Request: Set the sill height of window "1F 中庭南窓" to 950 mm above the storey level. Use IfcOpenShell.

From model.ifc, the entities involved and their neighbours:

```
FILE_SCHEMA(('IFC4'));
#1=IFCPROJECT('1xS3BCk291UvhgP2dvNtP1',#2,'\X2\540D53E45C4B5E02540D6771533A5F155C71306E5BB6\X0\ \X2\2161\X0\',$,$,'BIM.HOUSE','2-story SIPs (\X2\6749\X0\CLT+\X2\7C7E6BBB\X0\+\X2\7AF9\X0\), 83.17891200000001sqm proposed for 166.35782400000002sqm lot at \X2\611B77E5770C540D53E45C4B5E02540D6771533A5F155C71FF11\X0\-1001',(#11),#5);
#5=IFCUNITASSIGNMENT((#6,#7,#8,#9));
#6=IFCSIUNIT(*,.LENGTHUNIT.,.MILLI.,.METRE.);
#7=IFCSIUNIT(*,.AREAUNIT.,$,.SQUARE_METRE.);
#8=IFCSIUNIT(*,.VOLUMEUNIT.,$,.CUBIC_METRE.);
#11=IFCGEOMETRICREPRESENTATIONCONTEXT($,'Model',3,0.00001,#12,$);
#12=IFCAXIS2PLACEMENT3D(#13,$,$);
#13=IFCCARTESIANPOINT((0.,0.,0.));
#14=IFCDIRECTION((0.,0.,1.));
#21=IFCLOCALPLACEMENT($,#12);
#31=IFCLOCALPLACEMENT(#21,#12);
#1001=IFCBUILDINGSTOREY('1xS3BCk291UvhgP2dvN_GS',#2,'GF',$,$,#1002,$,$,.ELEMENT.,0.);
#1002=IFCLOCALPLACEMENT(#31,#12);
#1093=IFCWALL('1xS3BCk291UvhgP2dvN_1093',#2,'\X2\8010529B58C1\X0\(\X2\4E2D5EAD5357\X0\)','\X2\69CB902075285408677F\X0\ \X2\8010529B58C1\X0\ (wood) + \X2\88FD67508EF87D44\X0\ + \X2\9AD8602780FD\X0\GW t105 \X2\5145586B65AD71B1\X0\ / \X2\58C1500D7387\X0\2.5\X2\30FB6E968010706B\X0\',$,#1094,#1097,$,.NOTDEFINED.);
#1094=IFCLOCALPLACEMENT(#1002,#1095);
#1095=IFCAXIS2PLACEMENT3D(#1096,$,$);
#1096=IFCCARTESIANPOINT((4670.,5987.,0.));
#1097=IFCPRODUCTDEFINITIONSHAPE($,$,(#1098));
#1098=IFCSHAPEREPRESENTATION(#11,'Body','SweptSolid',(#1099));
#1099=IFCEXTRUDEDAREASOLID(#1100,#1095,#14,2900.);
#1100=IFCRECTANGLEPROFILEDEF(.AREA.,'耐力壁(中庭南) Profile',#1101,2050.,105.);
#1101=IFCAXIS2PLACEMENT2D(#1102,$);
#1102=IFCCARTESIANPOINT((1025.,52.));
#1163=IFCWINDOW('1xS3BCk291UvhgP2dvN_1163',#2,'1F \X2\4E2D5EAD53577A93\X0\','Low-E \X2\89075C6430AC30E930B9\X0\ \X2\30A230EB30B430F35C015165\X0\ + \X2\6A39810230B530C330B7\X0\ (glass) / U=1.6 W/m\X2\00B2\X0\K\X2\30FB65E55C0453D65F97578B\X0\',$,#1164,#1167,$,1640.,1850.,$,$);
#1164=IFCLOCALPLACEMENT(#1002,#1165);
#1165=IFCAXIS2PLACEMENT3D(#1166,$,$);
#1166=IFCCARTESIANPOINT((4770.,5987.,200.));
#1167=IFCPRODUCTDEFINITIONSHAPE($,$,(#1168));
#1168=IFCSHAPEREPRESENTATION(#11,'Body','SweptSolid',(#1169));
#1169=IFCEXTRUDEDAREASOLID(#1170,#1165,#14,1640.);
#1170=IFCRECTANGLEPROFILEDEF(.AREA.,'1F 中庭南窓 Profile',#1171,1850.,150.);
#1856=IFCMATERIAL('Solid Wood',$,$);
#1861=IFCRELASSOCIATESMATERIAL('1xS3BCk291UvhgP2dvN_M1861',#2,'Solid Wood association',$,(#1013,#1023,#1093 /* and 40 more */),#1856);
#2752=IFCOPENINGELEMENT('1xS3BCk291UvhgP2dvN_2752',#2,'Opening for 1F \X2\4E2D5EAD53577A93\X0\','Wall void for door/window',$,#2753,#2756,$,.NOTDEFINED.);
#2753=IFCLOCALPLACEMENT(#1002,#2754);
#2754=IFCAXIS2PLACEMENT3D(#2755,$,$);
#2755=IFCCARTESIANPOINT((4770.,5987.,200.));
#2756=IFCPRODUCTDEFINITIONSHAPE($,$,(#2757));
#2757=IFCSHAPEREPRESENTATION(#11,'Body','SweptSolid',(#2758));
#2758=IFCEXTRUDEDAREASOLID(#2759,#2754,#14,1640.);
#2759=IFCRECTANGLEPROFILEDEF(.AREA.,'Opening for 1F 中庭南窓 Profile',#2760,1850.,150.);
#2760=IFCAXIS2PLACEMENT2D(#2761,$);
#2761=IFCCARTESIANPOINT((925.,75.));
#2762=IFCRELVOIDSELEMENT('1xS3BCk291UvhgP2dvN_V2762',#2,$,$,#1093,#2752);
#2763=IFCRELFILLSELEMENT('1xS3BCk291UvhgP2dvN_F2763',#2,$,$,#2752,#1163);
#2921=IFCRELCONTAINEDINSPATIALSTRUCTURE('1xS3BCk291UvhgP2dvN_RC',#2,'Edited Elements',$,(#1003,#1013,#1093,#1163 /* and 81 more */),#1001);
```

```python
import numpy as np
import ifcopenshell
import ifcopenshell.api.geometry
import ifcopenshell.geom
import ifcopenshell.util.element
import ifcopenshell.util.placement
import ifcopenshell.util.shape
import ifcopenshell.util.unit

model = ifcopenshell.open("model.ifc")
unit_scale = ifcopenshell.util.unit.calculate_unit_scale(model)

window = model.by_id(1163)
opening = window.FillsVoids[0].RelatingOpeningElement
storey = ifcopenshell.util.element.get_container(window, ifc_class="IfcBuildingStorey")
level = ifcopenshell.util.placement.get_local_placement(storey.ObjectPlacement)[2, 3]

# The opening's origin need not be at the sill, so measure its lowest point.
shape = ifcopenshell.geom.create_shape(ifcopenshell.geom.settings(), opening)
bottom = ifcopenshell.util.shape.get_shape_bottom_elevation(shape, shape.geometry) / unit_scale
dz = level + 950.0 - bottom

shift = np.array([0.0, 0.0, dz])
# The window is not placed relative to its opening, so move both.
for product in (opening, window):
    matrix = ifcopenshell.util.placement.get_local_placement(product.ObjectPlacement)
    matrix[:3, 3] += shift
    ifcopenshell.api.geometry.edit_object_placement(model, product=product, matrix=matrix, is_si=False)

print(f"moved by {dz * unit_scale:+.3f} m")

model.write("model_v2.ifc")
```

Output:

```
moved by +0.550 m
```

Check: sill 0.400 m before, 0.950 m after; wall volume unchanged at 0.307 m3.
